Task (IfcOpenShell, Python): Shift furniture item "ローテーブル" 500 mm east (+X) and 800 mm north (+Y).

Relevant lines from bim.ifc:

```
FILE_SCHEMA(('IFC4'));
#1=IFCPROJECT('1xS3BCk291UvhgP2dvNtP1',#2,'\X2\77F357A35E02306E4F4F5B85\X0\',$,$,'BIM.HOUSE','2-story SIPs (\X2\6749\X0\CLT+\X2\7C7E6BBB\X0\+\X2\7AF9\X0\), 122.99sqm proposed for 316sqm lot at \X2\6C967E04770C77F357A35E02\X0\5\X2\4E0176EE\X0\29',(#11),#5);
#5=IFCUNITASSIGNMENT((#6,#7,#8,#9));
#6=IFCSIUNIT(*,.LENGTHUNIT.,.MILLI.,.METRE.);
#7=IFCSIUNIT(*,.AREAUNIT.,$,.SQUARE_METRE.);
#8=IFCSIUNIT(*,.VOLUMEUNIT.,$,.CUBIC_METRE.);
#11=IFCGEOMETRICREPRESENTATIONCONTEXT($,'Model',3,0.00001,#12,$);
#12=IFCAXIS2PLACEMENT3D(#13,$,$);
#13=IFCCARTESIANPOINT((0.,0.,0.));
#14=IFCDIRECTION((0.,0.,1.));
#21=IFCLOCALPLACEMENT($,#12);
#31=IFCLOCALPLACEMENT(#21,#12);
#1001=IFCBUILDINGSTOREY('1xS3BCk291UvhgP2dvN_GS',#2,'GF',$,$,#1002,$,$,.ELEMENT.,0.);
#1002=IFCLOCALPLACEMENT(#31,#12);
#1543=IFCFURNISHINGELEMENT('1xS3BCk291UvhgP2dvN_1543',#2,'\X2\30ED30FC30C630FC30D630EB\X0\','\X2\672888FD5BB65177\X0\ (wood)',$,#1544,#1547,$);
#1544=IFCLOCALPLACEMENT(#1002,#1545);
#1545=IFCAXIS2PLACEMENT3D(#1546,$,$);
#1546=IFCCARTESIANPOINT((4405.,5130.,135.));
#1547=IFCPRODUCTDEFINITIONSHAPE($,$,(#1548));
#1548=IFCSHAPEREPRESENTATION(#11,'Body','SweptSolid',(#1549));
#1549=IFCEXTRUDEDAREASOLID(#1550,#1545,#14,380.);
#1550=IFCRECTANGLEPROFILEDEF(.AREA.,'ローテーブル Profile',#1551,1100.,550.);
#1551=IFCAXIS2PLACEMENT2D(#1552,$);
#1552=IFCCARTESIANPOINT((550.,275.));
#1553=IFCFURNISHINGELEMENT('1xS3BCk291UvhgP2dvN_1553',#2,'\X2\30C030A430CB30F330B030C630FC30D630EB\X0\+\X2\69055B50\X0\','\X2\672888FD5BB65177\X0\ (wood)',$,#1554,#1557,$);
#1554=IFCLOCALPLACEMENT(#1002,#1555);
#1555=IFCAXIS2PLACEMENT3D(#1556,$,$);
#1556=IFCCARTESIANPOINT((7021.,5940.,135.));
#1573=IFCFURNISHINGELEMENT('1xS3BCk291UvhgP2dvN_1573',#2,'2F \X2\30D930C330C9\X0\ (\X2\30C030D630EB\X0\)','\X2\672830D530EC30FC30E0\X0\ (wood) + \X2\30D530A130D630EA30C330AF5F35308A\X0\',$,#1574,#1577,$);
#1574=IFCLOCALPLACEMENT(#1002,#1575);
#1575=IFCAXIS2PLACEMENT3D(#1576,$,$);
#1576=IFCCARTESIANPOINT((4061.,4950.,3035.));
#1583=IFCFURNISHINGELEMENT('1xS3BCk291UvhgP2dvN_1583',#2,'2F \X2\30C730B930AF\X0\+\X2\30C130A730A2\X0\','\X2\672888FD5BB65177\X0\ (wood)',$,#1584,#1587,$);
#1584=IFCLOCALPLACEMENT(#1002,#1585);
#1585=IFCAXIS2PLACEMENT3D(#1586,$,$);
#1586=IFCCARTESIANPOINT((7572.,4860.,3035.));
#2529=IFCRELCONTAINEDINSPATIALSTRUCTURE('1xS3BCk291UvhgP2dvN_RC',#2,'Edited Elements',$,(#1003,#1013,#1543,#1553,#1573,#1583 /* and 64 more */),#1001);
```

```python
import ifcopenshell
import ifcopenshell.api.geometry
import ifcopenshell.util.placement

model = ifcopenshell.open("bim.ifc")

item = model.by_id(1543)
matrix = ifcopenshell.util.placement.get_local_placement(item.ObjectPlacement)
matrix[0, 3] += 500.0
matrix[1, 3] += 800.0
ifcopenshell.api.geometry.edit_object_placement(model, product=item, matrix=matrix, is_si=False)

print(ifcopenshell.util.placement.get_local_placement(item.ObjectPlacement).round(3) + 0.0)

model.write("bim_rev.ifc")
```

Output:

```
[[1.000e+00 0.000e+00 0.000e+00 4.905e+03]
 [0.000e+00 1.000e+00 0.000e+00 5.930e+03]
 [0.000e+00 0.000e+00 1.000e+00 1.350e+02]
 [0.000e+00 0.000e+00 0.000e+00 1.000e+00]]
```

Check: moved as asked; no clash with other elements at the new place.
